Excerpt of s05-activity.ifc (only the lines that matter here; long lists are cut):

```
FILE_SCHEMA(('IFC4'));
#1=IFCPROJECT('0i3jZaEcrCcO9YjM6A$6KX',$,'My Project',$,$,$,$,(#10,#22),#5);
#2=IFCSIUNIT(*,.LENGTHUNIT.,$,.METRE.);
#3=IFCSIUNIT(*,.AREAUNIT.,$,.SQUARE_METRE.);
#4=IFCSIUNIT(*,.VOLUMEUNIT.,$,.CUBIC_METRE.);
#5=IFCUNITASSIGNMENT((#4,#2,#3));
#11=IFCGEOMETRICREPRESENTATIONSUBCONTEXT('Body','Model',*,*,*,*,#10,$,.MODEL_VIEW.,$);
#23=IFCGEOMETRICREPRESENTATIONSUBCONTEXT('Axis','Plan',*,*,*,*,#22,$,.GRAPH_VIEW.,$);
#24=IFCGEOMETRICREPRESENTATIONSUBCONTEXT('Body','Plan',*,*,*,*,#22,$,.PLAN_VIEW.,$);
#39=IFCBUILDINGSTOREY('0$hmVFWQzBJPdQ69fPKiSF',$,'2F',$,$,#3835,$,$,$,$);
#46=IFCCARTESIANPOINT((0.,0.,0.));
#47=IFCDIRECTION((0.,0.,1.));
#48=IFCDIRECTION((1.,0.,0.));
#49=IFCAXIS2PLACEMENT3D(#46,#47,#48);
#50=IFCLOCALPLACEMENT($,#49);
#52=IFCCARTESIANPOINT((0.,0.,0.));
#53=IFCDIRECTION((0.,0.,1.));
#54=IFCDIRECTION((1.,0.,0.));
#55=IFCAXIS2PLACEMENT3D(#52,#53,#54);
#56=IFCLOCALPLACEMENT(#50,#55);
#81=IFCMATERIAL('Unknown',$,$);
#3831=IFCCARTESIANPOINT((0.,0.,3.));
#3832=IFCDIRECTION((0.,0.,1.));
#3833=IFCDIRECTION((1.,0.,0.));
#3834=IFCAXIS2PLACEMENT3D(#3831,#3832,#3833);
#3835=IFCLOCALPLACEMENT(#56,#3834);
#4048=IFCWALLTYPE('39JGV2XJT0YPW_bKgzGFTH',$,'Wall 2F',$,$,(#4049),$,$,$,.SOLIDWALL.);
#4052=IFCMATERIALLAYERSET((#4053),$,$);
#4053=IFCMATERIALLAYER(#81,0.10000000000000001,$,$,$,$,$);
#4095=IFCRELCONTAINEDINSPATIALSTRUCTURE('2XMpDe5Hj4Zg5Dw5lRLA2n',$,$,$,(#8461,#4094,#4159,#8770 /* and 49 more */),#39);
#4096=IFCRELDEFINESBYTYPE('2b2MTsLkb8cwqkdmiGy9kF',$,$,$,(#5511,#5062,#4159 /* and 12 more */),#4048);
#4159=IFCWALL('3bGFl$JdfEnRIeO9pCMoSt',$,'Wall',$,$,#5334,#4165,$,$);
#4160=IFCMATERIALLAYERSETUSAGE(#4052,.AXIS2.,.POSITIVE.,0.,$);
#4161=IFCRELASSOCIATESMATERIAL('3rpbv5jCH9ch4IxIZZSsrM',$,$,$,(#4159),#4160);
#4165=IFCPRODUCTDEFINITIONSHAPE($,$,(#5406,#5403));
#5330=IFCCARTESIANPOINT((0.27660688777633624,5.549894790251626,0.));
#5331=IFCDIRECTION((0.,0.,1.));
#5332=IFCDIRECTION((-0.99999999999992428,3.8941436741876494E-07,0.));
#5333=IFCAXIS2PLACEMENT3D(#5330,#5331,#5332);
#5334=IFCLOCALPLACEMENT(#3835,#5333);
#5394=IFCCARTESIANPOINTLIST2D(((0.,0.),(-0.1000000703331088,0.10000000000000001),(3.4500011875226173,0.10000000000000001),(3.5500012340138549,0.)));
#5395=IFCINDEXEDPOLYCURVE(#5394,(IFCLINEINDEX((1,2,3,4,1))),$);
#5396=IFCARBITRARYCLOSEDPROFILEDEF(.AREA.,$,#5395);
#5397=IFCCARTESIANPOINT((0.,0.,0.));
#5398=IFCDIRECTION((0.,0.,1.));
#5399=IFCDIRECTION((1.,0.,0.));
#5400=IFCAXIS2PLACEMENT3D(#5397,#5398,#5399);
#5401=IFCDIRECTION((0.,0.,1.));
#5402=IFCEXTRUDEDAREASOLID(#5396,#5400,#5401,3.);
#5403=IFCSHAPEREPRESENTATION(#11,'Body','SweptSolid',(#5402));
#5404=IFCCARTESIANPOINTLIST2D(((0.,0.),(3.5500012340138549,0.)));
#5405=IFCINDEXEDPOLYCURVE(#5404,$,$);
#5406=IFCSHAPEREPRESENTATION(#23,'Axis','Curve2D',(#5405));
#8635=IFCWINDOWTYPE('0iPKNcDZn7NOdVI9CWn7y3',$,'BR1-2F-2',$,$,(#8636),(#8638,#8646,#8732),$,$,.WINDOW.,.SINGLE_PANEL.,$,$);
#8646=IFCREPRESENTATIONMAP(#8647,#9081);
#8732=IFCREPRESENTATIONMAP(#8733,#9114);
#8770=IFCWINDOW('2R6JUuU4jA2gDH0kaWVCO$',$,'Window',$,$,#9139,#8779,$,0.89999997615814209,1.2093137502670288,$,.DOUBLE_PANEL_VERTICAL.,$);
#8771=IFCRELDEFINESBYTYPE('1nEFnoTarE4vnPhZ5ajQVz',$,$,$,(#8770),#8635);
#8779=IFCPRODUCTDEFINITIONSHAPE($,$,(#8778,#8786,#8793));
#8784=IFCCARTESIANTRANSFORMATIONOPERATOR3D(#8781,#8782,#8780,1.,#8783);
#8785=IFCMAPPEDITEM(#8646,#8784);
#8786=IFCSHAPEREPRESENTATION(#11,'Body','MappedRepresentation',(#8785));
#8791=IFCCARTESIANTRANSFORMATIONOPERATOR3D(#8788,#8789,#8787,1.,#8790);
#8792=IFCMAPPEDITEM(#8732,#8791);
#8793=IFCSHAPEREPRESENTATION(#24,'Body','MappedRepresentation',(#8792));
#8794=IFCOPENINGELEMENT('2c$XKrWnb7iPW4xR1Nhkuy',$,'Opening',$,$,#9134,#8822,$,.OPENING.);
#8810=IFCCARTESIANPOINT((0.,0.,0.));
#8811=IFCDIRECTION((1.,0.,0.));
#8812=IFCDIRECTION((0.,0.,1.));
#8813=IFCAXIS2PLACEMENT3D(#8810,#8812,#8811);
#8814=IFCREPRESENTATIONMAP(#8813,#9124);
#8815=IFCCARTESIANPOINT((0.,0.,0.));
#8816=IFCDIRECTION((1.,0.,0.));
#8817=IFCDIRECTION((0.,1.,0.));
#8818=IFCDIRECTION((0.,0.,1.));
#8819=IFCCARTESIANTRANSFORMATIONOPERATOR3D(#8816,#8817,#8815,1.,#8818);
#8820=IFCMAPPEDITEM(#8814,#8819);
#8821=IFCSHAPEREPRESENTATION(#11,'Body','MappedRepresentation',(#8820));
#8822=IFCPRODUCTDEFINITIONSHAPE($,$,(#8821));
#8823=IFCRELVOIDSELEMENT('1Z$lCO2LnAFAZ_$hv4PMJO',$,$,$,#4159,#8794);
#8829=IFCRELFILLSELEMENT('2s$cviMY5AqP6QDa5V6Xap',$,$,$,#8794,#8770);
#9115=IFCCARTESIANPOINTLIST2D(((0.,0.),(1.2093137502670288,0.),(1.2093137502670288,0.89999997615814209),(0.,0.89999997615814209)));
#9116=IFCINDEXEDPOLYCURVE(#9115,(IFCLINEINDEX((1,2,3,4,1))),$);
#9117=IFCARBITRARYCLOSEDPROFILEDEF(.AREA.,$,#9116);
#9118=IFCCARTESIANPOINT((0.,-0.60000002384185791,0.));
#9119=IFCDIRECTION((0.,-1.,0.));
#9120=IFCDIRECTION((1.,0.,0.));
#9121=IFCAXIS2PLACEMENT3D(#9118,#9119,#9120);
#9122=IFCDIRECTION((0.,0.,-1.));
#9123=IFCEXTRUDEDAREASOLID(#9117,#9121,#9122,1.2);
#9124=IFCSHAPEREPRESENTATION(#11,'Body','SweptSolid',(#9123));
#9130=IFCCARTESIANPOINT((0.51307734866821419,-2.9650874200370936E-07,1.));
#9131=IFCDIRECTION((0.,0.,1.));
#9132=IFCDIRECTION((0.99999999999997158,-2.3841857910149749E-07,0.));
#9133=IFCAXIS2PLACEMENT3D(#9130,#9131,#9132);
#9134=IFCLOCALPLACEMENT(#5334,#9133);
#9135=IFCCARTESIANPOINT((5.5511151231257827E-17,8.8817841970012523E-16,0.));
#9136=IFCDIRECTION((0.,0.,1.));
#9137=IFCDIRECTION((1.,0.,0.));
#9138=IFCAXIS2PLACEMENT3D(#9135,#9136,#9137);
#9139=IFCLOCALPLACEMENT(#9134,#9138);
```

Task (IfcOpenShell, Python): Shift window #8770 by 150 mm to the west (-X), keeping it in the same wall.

```python
import ifcopenshell
import ifcopenshell.api.geometry
import ifcopenshell.util.placement
import ifcopenshell.util.unit

model = ifcopenshell.open("s05-activity.ifc")
unit_scale = ifcopenshell.util.unit.calculate_unit_scale(model)

window = model.by_id(8770)
opening = window.FillsVoids[0].RelatingOpeningElement
wall = opening.VoidsElements[0].RelatingBuildingElement

wall_matrix = ifcopenshell.util.placement.get_local_placement(wall.ObjectPlacement)
shift = wall_matrix[:3, 0] * 0.15 / unit_scale
before = ifcopenshell.util.placement.get_local_placement(window.ObjectPlacement)[:3, 3].copy()

# The window is placed relative to its opening, so it follows when the opening moves.
matrix = ifcopenshell.util.placement.get_local_placement(opening.ObjectPlacement)
matrix[:3, 3] += shift
ifcopenshell.api.geometry.edit_object_placement(
    model, product=opening, matrix=matrix, is_si=False, should_transform_children=True
)

after = ifcopenshell.util.placement.get_local_placement(window.ObjectPlacement)[:3, 3]
print("window moved by", (after - before).round(3) + 0.0)

model.write("s05-activity_edited.ifc")
```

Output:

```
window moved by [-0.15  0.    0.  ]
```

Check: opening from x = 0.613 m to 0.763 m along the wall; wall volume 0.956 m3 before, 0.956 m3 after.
